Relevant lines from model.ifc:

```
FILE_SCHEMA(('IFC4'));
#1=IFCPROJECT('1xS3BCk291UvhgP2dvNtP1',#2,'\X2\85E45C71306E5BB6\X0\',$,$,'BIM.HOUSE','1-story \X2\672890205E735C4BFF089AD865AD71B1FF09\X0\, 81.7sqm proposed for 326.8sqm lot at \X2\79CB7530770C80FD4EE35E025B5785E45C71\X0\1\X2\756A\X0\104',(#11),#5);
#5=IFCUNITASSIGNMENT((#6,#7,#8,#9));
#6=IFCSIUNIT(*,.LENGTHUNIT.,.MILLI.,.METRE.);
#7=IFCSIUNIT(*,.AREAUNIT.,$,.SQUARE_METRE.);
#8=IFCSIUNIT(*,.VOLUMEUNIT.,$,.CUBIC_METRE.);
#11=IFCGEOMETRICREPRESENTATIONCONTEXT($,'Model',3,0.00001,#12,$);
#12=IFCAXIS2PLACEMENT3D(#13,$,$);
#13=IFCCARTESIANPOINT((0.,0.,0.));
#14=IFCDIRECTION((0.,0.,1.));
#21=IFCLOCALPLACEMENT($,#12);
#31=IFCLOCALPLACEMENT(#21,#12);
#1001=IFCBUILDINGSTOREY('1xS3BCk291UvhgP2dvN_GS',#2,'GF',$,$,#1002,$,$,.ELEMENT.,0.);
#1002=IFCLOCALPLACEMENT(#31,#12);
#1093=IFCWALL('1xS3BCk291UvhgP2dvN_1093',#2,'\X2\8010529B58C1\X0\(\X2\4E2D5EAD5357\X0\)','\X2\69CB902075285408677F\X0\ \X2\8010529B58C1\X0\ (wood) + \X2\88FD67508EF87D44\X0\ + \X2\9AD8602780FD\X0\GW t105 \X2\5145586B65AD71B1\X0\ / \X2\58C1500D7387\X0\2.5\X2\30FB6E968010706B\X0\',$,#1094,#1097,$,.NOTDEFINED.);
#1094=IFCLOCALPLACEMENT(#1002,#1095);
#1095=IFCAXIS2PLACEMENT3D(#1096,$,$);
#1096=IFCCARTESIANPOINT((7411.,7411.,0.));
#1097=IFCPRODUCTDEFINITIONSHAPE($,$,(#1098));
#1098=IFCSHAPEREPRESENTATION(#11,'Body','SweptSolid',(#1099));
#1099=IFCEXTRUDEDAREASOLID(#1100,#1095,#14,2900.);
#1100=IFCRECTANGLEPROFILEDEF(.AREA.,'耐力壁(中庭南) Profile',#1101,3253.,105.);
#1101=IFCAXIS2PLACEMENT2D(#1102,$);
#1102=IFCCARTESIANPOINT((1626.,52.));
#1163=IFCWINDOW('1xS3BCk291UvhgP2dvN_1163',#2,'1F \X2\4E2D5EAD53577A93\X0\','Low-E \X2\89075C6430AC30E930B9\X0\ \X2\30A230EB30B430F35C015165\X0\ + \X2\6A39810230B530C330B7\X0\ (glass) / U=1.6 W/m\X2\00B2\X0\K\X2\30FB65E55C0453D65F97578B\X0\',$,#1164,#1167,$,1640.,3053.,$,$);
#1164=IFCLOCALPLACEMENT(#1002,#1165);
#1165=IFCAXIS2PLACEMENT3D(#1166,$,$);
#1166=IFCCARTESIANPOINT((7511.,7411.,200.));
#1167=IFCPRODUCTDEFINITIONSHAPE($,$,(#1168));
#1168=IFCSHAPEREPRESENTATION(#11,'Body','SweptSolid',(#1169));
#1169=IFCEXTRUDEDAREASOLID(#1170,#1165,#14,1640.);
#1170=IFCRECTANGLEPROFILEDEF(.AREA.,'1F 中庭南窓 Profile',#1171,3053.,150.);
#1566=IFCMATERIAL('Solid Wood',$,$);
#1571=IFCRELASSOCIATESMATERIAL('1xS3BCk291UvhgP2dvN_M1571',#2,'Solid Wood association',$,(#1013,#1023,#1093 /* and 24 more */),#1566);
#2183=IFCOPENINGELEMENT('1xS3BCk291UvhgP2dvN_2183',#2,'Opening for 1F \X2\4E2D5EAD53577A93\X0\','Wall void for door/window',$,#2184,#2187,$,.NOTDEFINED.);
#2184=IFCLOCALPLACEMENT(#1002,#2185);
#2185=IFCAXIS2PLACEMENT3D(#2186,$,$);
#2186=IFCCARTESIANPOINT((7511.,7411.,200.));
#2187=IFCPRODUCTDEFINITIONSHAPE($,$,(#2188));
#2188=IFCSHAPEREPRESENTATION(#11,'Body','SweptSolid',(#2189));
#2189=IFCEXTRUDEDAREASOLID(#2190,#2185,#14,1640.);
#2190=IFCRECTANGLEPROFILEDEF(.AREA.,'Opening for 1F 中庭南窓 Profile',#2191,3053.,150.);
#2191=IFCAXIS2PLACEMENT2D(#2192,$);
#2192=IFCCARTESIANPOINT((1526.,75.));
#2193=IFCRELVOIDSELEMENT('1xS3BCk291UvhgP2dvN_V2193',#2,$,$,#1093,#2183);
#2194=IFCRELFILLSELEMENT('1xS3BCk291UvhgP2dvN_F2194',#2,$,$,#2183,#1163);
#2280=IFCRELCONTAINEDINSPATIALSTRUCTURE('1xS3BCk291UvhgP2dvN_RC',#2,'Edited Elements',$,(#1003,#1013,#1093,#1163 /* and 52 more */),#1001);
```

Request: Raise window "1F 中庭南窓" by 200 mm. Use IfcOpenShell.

```python
import numpy as np
import ifcopenshell
import ifcopenshell.api.geometry
import ifcopenshell.util.placement
import ifcopenshell.util.unit

model = ifcopenshell.open("model.ifc")
unit_scale = ifcopenshell.util.unit.calculate_unit_scale(model)

window = model.by_guid("1xS3BCk291UvhgP2dvN_1163")
opening = window.FillsVoids[0].RelatingOpeningElement
dz = 0.2 / unit_scale

shift = np.array([0.0, 0.0, dz])
# The window is not placed relative to its opening, so move both.
for product in (opening, window):
    matrix = ifcopenshell.util.placement.get_local_placement(product.ObjectPlacement)
    matrix[:3, 3] += shift
    ifcopenshell.api.geometry.edit_object_placement(model, product=product, matrix=matrix, is_si=False)

print(f"moved by {dz * unit_scale:+.3f} m")

model.write("model-out.ifc")
```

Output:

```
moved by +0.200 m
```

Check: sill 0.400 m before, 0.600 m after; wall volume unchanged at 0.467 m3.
